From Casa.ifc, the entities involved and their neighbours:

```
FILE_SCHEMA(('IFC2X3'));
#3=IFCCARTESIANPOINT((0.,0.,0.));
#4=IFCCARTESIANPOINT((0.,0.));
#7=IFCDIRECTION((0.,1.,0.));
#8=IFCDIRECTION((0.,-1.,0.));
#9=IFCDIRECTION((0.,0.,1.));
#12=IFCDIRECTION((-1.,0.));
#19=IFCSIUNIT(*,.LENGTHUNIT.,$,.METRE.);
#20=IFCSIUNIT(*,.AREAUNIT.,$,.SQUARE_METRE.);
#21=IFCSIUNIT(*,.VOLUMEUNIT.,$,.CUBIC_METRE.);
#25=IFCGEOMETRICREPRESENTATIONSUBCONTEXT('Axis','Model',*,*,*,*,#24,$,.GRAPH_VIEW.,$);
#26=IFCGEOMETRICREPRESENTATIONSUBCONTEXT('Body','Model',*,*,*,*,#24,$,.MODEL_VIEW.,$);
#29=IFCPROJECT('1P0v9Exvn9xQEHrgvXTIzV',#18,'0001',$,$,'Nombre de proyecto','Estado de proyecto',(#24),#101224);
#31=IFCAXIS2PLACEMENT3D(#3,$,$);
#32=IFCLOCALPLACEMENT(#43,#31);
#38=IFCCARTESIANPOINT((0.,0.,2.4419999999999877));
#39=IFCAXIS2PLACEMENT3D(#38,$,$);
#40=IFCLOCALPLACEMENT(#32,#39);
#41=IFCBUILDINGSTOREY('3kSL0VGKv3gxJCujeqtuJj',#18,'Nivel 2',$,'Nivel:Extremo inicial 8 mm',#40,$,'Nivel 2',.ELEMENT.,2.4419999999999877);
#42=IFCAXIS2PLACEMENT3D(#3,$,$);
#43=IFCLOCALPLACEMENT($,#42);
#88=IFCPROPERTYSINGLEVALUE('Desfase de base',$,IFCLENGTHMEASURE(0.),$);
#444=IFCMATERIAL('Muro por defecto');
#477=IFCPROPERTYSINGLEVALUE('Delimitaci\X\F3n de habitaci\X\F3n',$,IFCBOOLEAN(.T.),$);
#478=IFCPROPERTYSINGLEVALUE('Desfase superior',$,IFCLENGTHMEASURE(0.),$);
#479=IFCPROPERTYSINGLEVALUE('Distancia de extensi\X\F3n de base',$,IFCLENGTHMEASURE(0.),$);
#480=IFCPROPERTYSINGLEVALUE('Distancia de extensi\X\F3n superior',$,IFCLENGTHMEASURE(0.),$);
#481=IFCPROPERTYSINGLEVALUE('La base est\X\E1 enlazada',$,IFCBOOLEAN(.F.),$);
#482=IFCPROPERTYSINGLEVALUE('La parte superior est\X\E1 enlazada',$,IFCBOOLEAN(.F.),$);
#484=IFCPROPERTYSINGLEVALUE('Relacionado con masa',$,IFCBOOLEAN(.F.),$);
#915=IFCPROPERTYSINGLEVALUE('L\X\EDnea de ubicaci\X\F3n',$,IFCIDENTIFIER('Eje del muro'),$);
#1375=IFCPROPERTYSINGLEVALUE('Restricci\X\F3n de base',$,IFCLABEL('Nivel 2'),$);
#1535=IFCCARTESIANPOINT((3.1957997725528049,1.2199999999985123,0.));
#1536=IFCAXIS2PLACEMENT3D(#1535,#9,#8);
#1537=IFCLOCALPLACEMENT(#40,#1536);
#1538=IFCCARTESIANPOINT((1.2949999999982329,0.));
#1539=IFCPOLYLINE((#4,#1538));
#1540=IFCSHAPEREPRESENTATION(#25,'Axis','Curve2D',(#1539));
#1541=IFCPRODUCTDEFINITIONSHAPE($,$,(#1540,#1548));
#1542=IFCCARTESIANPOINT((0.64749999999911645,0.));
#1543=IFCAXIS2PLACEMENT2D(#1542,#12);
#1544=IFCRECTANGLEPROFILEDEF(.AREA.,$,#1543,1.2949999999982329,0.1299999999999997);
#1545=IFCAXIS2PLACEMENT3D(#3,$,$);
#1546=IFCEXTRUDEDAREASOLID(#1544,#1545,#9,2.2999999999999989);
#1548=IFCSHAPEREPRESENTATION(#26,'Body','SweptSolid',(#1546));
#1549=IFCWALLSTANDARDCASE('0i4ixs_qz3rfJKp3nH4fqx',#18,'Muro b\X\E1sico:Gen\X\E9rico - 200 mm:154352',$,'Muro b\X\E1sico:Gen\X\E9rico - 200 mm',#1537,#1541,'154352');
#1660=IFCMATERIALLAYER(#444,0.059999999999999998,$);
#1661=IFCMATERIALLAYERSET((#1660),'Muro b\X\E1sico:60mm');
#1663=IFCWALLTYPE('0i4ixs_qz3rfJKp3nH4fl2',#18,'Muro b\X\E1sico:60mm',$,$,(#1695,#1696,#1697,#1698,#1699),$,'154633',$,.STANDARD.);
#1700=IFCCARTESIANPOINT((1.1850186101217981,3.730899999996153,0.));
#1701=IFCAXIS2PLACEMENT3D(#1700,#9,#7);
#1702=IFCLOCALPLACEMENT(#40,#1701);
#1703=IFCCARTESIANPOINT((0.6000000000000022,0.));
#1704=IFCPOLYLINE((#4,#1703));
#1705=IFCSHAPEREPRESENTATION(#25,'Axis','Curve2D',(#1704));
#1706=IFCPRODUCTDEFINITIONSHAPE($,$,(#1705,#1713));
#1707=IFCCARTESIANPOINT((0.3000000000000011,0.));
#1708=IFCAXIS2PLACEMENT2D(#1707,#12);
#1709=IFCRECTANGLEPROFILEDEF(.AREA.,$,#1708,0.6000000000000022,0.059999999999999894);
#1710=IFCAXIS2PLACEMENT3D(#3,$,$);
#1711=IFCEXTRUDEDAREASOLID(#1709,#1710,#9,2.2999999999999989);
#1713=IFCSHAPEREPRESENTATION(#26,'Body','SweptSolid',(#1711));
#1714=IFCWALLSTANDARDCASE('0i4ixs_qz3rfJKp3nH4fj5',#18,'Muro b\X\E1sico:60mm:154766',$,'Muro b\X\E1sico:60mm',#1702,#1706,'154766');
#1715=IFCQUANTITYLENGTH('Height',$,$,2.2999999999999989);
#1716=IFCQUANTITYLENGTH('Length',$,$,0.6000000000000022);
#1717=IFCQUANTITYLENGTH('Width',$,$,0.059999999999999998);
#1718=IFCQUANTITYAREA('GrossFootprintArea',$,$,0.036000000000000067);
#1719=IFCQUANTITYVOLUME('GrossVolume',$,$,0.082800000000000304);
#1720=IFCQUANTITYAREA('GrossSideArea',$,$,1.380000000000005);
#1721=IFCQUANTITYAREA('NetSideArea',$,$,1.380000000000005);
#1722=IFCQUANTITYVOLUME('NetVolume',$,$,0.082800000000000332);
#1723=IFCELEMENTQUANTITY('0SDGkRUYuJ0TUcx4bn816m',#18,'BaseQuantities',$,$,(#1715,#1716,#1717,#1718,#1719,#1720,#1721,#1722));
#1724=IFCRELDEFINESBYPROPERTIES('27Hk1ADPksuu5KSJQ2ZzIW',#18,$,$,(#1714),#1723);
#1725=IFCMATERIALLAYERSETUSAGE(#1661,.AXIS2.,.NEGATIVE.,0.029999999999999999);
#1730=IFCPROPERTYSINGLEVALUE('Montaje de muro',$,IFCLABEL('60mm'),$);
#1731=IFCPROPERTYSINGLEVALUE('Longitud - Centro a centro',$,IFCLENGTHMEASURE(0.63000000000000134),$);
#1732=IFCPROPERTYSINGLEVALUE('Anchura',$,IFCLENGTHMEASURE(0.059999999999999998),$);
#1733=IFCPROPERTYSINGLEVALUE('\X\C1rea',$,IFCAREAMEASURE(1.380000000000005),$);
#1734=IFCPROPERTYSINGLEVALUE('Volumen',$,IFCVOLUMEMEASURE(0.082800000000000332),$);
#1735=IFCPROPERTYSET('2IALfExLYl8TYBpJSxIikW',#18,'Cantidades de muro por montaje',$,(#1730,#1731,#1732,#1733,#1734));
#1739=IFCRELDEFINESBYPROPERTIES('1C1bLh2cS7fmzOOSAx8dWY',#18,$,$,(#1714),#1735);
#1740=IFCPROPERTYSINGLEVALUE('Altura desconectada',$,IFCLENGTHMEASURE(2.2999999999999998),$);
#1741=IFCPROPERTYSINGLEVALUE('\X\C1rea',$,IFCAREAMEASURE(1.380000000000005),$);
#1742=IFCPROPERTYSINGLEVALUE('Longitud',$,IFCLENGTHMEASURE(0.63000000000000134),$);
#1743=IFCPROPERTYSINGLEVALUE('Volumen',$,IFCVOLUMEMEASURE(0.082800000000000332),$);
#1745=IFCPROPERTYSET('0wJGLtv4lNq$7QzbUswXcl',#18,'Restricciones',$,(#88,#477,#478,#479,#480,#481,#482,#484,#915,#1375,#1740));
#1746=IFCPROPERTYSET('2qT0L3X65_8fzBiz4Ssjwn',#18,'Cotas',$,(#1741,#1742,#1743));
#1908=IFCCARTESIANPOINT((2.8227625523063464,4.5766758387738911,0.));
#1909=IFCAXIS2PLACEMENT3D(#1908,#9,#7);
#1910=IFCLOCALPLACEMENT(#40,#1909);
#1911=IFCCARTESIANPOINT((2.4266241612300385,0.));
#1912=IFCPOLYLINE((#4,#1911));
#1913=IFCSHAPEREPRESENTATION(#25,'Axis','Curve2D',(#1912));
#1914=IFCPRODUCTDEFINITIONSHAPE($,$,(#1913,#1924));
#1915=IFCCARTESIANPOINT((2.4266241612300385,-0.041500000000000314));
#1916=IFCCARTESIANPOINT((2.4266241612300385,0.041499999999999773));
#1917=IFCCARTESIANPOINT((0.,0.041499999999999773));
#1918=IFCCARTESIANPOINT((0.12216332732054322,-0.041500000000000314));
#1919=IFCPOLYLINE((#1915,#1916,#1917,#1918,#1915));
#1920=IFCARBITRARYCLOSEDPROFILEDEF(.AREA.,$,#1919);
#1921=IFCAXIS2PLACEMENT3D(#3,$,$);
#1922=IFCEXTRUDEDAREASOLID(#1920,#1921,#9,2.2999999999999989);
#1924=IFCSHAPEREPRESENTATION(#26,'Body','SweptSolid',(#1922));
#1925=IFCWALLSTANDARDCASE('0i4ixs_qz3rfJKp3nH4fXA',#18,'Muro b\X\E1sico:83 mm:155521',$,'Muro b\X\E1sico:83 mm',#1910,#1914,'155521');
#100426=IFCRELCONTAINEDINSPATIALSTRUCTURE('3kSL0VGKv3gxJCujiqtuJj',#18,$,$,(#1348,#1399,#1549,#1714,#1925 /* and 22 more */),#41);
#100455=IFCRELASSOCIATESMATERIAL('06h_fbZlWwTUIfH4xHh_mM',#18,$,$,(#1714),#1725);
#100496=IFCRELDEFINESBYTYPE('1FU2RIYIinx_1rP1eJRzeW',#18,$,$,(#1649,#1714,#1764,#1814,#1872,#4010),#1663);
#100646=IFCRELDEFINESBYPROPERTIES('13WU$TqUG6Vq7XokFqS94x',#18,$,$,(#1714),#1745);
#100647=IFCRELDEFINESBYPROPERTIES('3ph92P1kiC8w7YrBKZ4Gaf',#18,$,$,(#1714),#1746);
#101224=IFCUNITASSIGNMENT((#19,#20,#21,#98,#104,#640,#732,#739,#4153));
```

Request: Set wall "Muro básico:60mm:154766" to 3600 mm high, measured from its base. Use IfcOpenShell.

```python
import ifcopenshell
import ifcopenshell.api.pset
import ifcopenshell.geom
import ifcopenshell.util.element
import ifcopenshell.util.representation
import ifcopenshell.util.shape
import ifcopenshell.util.unit

model = ifcopenshell.open("Casa.ifc")
unit_scale = ifcopenshell.util.unit.calculate_unit_scale(model)
area_scale = ifcopenshell.util.unit.calculate_unit_scale(model, "AREAUNIT")
volume_scale = ifcopenshell.util.unit.calculate_unit_scale(model, "VOLUMEUNIT")
settings = ifcopenshell.geom.settings()


def volume(element):
    """Net volume in cubic metres, openings subtracted."""
    shape = ifcopenshell.geom.create_shape(settings, element)
    return ifcopenshell.util.shape.get_volume(shape.geometry)


wall = model.by_id(1714)
before = volume(wall)

body = ifcopenshell.util.representation.get_representation(wall, "Model", "Body")
solid = body.Items[0]
old_height = solid.Depth
solid.Depth = 3.6 / unit_scale
after = volume(wall)
thickness = 0.06  # wall thickness in metres

# Update the stored height, areas and volumes.
qto = model.by_id(ifcopenshell.util.element.get_pset(wall, "BaseQuantities", should_inherit=False)["id"])
ifcopenshell.api.pset.edit_qto(model, qto=qto, properties={
    "Height": solid.Depth,
    "GrossVolume": ifcopenshell.util.element.get_pset(wall, "BaseQuantities", "GrossVolume") * solid.Depth / old_height,
    "GrossSideArea": ifcopenshell.util.element.get_pset(wall, "BaseQuantities", "GrossSideArea") * solid.Depth / old_height,
    "NetSideArea": after / thickness / area_scale,
    "NetVolume": after / volume_scale,
})
pset = model.by_id(ifcopenshell.util.element.get_pset(wall, "Cantidades de muro por montaje", should_inherit=False)["id"])
ifcopenshell.api.pset.edit_pset(model, pset=pset, properties={
    "Área": model.create_entity("IfcAreaMeasure", after / thickness / area_scale),
    "Volumen": model.create_entity("IfcVolumeMeasure", after / volume_scale),
})
pset = model.by_id(ifcopenshell.util.element.get_pset(wall, "Restricciones", should_inherit=False)["id"])
ifcopenshell.api.pset.edit_pset(model, pset=pset, properties={
    "Altura desconectada": model.create_entity("IfcLengthMeasure", solid.Depth),
})
pset = model.by_id(ifcopenshell.util.element.get_pset(wall, "Cotas", should_inherit=False)["id"])
ifcopenshell.api.pset.edit_pset(model, pset=pset, properties={
    "Área": model.create_entity("IfcAreaMeasure", after / thickness / area_scale),
    "Volumen": model.create_entity("IfcVolumeMeasure", after / volume_scale),
})

print(f"height {old_height:g} -> {solid.Depth:g}, volume {before:.3f} -> {after:.3f} m3")

model.write("Casa-out.ifc")
```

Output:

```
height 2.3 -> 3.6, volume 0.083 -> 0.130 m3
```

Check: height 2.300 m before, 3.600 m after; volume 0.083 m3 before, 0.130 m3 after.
